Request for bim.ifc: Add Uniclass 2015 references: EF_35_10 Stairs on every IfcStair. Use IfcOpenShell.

First a look at what the model holds.

```python
import ifcopenshell

model = ifcopenshell.open("bim.ifc")
print(model.schema)
print("classifications:", [c.Name for c in model.by_type("IfcClassification")])
for ifc_class in ("IfcDoor", "IfcRoof", "IfcStair", "IfcWall", "IfcWindow"):
    print(ifc_class, len(model.by_type(ifc_class)))
```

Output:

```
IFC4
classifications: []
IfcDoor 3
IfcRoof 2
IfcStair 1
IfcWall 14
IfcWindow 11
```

```python
import ifcopenshell
import ifcopenshell.api.classification

model = ifcopenshell.open("bim.ifc")

system = ifcopenshell.api.classification.add_classification(model, classification="Uniclass 2015")

codes = {
    "IfcStair": ("EF_35_10", "Stairs"),
}
for ifc_class, (code, name) in codes.items():
    products = model.by_type(ifc_class)
    ifcopenshell.api.classification.add_reference(
        model, products=products, classification=system, identification=code, name=name
    )
    print(code, len(products))

model.write("bim-out.ifc")
```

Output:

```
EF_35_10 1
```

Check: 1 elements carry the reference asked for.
